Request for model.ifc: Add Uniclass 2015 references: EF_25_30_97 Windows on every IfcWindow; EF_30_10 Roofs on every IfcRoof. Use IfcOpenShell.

First a look at what the model holds.

```python
import ifcopenshell

model = ifcopenshell.open("model.ifc")
print(model.schema)
print("classifications:", [c.Name for c in model.by_type("IfcClassification")])
for ifc_class in ("IfcDoor", "IfcRoof", "IfcStair", "IfcWall", "IfcWindow"):
    print(ifc_class, len(model.by_type(ifc_class)))
```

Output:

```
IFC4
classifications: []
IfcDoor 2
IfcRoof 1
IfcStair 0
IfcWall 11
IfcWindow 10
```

```python
import ifcopenshell
import ifcopenshell.api.classification

model = ifcopenshell.open("model.ifc")

system = ifcopenshell.api.classification.add_classification(model, classification="Uniclass 2015")

codes = {
    "IfcWindow": ("EF_25_30_97", "Windows"),
    "IfcRoof": ("EF_30_10", "Roofs"),
}
for ifc_class, (code, name) in codes.items():
    products = model.by_type(ifc_class)
    ifcopenshell.api.classification.add_reference(
        model, products=products, classification=system, identification=code, name=name
    )
    print(code, len(products))

model.write("model-out.ifc")
```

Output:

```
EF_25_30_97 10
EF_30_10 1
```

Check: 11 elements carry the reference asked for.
